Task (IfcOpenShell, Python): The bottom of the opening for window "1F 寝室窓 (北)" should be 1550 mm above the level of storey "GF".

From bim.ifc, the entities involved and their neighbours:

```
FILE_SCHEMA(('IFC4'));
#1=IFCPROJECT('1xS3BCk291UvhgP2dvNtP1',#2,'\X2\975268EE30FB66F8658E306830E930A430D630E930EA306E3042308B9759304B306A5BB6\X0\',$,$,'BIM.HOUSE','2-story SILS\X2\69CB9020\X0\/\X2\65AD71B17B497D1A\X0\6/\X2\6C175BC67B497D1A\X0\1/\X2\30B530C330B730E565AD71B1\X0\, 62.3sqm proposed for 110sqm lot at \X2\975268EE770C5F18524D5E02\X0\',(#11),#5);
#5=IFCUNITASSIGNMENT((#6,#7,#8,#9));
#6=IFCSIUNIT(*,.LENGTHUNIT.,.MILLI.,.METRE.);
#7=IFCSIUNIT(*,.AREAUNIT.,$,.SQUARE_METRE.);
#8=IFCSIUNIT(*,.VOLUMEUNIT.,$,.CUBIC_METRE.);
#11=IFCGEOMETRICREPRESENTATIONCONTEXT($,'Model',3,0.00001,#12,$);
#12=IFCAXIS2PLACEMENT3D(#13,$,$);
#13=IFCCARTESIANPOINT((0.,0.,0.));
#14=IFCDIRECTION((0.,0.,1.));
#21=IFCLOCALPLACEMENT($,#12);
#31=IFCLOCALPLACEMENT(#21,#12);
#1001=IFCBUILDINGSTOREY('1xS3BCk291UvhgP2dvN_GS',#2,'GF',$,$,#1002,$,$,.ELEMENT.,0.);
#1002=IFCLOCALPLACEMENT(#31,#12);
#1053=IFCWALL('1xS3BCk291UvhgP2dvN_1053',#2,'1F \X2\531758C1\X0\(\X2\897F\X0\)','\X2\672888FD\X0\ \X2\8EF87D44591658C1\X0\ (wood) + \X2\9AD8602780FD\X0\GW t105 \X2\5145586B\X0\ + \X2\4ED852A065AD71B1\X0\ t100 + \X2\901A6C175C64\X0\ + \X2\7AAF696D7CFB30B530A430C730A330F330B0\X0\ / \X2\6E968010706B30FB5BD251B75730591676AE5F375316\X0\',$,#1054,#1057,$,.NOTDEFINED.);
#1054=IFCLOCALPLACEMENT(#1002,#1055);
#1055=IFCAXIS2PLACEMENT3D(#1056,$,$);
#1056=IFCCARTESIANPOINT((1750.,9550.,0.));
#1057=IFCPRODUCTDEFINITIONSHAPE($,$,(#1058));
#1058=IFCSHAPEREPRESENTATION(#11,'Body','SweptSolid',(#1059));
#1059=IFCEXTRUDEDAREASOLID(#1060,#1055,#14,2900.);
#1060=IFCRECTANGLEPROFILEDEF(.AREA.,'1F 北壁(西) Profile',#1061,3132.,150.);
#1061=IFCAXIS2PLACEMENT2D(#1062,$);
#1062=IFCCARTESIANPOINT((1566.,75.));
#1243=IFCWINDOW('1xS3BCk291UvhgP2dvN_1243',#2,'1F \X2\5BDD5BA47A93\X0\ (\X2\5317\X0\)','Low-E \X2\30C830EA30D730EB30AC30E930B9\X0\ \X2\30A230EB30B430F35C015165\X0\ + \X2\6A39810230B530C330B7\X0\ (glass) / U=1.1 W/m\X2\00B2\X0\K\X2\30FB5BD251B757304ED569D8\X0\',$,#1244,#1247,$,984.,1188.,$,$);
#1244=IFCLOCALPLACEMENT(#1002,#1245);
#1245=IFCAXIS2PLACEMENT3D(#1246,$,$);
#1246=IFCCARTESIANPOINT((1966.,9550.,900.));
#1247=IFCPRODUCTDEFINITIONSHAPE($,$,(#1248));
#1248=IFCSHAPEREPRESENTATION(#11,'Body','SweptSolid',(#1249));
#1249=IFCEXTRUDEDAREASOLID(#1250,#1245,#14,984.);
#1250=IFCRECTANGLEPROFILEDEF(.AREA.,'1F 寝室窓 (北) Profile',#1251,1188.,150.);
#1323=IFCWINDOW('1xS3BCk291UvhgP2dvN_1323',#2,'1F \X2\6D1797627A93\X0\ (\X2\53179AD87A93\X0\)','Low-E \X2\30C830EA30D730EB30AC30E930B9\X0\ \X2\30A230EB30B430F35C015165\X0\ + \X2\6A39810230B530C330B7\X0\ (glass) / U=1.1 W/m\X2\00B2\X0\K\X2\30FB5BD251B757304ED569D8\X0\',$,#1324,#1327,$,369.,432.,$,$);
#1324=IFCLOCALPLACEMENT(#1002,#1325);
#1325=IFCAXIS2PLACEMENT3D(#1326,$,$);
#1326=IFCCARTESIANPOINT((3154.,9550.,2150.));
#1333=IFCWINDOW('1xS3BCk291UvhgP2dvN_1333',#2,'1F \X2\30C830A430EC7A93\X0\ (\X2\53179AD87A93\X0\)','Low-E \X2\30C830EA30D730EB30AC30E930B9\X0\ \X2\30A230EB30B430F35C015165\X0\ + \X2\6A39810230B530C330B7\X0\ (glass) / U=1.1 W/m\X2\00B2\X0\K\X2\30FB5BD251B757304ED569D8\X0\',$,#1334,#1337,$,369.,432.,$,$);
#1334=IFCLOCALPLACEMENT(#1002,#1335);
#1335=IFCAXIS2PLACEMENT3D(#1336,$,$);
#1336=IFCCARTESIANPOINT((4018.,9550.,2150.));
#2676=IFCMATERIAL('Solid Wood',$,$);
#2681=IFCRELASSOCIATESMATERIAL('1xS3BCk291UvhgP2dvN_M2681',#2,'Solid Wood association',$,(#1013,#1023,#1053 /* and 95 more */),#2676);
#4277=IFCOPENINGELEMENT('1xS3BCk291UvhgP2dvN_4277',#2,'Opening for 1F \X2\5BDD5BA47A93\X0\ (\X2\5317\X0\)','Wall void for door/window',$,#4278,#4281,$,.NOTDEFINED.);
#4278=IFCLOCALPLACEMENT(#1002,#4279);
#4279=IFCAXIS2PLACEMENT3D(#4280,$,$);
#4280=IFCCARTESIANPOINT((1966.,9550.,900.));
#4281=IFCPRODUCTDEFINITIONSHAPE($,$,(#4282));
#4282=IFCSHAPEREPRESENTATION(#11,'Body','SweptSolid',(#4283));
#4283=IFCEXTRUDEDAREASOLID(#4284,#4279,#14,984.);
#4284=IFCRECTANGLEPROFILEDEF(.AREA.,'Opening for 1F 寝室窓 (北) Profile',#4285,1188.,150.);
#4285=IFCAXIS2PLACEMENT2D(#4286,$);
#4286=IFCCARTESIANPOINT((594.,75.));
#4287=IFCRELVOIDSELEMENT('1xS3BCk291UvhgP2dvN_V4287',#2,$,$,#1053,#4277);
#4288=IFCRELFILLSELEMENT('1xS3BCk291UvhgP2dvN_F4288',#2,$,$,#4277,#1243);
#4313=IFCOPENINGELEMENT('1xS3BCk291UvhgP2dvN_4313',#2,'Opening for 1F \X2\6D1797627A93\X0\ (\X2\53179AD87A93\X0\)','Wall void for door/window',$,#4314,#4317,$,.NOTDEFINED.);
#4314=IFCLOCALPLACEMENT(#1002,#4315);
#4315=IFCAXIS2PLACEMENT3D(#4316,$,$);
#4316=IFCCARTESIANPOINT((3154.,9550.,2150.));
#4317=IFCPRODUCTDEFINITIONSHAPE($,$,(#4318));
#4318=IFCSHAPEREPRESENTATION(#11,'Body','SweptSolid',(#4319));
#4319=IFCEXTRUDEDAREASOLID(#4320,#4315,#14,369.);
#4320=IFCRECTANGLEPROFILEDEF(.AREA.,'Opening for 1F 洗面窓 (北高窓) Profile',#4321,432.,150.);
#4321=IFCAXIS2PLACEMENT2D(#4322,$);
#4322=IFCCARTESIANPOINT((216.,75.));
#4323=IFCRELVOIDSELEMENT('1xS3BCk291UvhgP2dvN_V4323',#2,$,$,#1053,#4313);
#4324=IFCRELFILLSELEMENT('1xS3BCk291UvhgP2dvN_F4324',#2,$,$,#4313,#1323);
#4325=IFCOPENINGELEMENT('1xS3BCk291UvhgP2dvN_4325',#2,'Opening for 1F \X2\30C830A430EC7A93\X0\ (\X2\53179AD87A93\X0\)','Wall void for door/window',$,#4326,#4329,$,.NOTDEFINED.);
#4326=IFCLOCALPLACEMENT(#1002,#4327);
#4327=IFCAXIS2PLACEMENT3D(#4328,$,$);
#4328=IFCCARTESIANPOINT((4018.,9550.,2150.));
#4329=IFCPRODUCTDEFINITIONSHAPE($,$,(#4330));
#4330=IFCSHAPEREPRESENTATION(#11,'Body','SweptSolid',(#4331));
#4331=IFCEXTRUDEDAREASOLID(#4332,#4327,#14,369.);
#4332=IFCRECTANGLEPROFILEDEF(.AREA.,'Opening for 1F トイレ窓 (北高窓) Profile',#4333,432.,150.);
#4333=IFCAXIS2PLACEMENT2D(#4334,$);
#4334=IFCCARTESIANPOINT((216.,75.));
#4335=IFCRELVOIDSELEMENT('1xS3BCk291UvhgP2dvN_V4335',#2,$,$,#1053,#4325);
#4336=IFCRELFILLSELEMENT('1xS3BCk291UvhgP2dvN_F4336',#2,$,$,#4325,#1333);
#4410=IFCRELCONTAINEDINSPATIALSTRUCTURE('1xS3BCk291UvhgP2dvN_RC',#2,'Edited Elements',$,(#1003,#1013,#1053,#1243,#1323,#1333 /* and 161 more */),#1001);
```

```python
import numpy as np
import ifcopenshell
import ifcopenshell.api.geometry
import ifcopenshell.geom
import ifcopenshell.util.element
import ifcopenshell.util.placement
import ifcopenshell.util.shape
import ifcopenshell.util.unit

model = ifcopenshell.open("bim.ifc")
unit_scale = ifcopenshell.util.unit.calculate_unit_scale(model)

window = model.by_guid("1xS3BCk291UvhgP2dvN_1243")
opening = window.FillsVoids[0].RelatingOpeningElement
storey = ifcopenshell.util.element.get_container(window, ifc_class="IfcBuildingStorey")
level = ifcopenshell.util.placement.get_local_placement(storey.ObjectPlacement)[2, 3]

# The opening's origin need not be at the sill, so measure its lowest point.
shape = ifcopenshell.geom.create_shape(ifcopenshell.geom.settings(), opening)
bottom = ifcopenshell.util.shape.get_shape_bottom_elevation(shape, shape.geometry) / unit_scale
dz = level + 1.55 / unit_scale - bottom

shift = np.array([0.0, 0.0, dz])
# The window is not placed relative to its opening, so move both.
for product in (opening, window):
    matrix = ifcopenshell.util.placement.get_local_placement(product.ObjectPlacement)
    matrix[:3, 3] += shift
    ifcopenshell.api.geometry.edit_object_placement(model, product=product, matrix=matrix, is_si=False)

print(f"moved by {dz * unit_scale:+.3f} m")

model.write("bim_edited.ifc")
```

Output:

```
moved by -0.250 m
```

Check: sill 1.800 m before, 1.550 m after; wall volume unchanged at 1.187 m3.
